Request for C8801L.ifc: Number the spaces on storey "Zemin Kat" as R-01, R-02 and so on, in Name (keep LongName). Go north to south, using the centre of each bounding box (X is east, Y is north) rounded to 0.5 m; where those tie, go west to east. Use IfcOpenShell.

First a look at what the model holds.

```python
import ifcopenshell
import ifcopenshell.util.element
import ifcopenshell.util.placement

model = ifcopenshell.open("C8801L.ifc")
print(model.schema)
storey = next(s for s in model.by_type("IfcBuildingStorey") if s.Name == "Zemin Kat")
spaces = [e for e in ifcopenshell.util.element.get_decomposition(storey) if e.is_a("IfcSpace")]
for e in sorted(spaces, key=lambda e: e.id()):
    origin = ifcopenshell.util.placement.get_local_placement(e.ObjectPlacement)[:3, 3]
    print(e.id(), e.Name, e.LongName, origin.round(2) + 0.0, sep=" | ")
```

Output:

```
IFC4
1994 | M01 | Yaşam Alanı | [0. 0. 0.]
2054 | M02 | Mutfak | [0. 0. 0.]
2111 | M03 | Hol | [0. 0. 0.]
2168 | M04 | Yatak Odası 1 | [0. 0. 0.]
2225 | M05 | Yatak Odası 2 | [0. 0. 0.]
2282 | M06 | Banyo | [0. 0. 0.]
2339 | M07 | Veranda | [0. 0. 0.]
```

```python
import ifcopenshell
import ifcopenshell.geom
import ifcopenshell.util.element
import ifcopenshell.util.shape

model = ifcopenshell.open("C8801L.ifc")
settings = ifcopenshell.geom.settings()
settings.set("use-world-coords", True)


def centre(element):
    shape = ifcopenshell.geom.create_shape(settings, element)
    return ifcopenshell.util.shape.get_bbox_centroid(shape.geometry)


storey = next(s for s in model.by_type("IfcBuildingStorey") if s.Name == "Zemin Kat")
spaces = [e for e in ifcopenshell.util.element.get_decomposition(storey) if e.is_a("IfcSpace")]

# Insertion points can sit at a corner or the storey origin, so sort by the geometry (in metres).
centres = {e: centre(e) for e in spaces}
spaces.sort(key=lambda e: (-round(centres[e][1] / 0.5), centres[e][0]))

for i, e in enumerate(spaces, start=1):
    number = f"R-{i:02d}"
    e.Name = number
    print(e.id(), number)

model.write("C8801L-out.ifc")
```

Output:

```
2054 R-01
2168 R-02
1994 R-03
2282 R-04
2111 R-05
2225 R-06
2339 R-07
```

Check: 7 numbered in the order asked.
